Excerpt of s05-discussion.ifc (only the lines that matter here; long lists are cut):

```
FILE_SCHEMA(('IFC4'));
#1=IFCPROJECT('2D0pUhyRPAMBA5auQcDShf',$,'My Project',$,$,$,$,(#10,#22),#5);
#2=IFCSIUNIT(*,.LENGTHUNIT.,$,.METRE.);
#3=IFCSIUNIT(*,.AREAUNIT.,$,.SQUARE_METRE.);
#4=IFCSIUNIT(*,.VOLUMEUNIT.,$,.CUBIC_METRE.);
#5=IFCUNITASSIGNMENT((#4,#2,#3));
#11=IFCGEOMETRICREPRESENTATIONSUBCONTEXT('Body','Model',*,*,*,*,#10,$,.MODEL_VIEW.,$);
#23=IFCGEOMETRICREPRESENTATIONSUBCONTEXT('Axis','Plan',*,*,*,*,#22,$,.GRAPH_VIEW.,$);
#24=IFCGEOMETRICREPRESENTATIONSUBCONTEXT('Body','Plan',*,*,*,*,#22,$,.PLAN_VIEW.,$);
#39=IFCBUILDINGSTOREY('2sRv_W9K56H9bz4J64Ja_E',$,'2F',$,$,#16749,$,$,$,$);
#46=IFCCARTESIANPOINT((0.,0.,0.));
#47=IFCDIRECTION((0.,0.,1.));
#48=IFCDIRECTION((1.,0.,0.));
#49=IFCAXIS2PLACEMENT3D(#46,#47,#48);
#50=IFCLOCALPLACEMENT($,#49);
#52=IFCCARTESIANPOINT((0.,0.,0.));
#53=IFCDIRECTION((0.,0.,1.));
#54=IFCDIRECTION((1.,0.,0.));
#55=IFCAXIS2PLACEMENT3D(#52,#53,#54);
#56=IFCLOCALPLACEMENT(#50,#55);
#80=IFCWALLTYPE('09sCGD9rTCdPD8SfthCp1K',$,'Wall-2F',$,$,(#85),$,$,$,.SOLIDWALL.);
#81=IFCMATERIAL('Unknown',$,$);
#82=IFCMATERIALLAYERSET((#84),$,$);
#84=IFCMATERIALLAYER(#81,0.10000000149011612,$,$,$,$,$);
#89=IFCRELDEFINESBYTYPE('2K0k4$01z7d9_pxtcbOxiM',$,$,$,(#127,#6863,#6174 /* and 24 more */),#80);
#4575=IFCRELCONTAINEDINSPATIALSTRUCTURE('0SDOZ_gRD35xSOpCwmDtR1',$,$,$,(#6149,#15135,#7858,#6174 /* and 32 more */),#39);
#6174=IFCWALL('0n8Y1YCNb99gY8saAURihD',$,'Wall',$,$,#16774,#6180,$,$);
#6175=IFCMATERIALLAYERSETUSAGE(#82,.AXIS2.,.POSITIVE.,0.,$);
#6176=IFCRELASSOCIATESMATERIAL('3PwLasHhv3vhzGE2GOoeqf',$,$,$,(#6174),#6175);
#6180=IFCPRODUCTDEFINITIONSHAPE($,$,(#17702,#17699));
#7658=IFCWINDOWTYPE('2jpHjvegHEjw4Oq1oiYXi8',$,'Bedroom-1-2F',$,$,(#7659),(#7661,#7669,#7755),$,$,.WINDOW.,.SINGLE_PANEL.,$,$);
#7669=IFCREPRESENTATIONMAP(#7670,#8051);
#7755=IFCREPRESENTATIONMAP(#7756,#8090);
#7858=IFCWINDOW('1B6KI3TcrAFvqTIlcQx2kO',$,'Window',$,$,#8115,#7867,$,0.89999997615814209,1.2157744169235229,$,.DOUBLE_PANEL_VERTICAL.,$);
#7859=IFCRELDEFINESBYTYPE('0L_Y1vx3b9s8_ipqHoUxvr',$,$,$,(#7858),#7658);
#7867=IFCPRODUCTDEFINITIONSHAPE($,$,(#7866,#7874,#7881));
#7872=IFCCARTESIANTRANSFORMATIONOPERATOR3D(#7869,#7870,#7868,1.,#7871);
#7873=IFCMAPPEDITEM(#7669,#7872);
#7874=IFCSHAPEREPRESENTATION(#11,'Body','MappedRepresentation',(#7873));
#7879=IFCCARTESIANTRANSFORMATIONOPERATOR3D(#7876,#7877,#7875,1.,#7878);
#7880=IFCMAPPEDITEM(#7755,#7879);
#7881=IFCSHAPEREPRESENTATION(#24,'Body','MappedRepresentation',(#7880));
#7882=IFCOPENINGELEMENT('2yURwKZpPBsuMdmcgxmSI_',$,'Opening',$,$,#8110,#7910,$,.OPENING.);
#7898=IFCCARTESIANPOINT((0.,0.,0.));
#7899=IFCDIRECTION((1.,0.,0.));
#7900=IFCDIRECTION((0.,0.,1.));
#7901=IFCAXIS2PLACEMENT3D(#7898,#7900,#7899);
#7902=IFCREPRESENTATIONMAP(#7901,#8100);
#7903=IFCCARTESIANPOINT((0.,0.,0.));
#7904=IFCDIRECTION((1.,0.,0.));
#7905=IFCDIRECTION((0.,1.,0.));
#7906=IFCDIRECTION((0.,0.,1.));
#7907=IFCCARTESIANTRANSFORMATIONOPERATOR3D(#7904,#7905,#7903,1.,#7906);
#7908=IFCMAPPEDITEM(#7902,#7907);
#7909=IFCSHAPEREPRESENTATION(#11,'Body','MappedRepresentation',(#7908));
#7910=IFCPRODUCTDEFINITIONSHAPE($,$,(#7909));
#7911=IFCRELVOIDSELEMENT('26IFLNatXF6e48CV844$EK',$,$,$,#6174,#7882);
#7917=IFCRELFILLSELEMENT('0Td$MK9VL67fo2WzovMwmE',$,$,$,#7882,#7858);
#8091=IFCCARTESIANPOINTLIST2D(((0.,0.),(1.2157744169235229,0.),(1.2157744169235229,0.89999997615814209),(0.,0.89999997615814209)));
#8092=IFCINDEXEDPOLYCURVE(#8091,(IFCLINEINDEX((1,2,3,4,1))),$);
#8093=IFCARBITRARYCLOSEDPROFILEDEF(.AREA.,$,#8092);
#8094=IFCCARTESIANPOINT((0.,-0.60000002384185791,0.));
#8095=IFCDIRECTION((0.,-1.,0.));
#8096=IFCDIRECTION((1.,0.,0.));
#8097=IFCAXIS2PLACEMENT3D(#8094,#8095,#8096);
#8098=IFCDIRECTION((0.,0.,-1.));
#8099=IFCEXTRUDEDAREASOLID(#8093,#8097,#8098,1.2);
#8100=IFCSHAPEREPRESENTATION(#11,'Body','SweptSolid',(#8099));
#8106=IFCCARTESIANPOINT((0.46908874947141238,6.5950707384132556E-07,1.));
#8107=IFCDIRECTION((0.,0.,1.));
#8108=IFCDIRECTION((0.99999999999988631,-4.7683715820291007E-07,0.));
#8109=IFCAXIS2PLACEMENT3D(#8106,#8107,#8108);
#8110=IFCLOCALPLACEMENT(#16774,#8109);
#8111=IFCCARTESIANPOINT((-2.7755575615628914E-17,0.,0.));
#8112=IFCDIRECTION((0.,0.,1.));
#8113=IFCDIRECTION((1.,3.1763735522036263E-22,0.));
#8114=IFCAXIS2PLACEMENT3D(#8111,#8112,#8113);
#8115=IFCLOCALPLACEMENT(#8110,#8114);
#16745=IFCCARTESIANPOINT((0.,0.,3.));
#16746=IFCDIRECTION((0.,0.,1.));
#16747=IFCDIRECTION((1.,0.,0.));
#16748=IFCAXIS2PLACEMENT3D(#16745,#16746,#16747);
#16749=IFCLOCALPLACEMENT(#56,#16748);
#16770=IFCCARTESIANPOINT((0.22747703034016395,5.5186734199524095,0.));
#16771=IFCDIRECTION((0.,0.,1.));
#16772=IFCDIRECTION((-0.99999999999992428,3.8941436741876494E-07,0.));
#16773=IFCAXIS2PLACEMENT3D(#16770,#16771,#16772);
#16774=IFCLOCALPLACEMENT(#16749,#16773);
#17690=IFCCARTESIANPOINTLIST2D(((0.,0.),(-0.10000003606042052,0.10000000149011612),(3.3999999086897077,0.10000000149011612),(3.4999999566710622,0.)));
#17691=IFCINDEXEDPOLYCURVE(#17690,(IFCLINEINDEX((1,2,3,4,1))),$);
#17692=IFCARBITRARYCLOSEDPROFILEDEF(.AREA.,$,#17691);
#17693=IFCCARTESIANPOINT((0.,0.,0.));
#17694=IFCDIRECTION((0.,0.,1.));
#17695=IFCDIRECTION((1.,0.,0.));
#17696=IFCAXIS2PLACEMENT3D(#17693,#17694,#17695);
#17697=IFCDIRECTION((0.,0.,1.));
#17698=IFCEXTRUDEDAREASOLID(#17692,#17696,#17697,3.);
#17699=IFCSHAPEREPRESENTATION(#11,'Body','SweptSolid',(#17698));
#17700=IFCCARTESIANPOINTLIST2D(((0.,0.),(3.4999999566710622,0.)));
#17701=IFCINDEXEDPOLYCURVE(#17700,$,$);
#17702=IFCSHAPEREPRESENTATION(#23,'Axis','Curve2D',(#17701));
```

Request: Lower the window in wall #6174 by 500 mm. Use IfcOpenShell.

```python
import numpy as np
import ifcopenshell
import ifcopenshell.api.geometry
import ifcopenshell.util.placement
import ifcopenshell.util.unit

model = ifcopenshell.open("s05-discussion.ifc")
unit_scale = ifcopenshell.util.unit.calculate_unit_scale(model)

window = model.by_guid("1B6KI3TcrAFvqTIlcQx2kO")
opening = window.FillsVoids[0].RelatingOpeningElement
dz = -0.5 / unit_scale

shift = np.array([0.0, 0.0, dz])
# The window is placed relative to its opening, so it follows when the opening moves.
matrix = ifcopenshell.util.placement.get_local_placement(opening.ObjectPlacement)
matrix[:3, 3] += shift
ifcopenshell.api.geometry.edit_object_placement(
    model, product=opening, matrix=matrix, is_si=False, should_transform_children=True
)

print(f"moved by {dz * unit_scale:+.3f} m")

model.write("s05-discussion_v2.ifc")
```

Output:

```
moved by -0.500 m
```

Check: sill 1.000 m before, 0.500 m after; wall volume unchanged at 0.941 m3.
